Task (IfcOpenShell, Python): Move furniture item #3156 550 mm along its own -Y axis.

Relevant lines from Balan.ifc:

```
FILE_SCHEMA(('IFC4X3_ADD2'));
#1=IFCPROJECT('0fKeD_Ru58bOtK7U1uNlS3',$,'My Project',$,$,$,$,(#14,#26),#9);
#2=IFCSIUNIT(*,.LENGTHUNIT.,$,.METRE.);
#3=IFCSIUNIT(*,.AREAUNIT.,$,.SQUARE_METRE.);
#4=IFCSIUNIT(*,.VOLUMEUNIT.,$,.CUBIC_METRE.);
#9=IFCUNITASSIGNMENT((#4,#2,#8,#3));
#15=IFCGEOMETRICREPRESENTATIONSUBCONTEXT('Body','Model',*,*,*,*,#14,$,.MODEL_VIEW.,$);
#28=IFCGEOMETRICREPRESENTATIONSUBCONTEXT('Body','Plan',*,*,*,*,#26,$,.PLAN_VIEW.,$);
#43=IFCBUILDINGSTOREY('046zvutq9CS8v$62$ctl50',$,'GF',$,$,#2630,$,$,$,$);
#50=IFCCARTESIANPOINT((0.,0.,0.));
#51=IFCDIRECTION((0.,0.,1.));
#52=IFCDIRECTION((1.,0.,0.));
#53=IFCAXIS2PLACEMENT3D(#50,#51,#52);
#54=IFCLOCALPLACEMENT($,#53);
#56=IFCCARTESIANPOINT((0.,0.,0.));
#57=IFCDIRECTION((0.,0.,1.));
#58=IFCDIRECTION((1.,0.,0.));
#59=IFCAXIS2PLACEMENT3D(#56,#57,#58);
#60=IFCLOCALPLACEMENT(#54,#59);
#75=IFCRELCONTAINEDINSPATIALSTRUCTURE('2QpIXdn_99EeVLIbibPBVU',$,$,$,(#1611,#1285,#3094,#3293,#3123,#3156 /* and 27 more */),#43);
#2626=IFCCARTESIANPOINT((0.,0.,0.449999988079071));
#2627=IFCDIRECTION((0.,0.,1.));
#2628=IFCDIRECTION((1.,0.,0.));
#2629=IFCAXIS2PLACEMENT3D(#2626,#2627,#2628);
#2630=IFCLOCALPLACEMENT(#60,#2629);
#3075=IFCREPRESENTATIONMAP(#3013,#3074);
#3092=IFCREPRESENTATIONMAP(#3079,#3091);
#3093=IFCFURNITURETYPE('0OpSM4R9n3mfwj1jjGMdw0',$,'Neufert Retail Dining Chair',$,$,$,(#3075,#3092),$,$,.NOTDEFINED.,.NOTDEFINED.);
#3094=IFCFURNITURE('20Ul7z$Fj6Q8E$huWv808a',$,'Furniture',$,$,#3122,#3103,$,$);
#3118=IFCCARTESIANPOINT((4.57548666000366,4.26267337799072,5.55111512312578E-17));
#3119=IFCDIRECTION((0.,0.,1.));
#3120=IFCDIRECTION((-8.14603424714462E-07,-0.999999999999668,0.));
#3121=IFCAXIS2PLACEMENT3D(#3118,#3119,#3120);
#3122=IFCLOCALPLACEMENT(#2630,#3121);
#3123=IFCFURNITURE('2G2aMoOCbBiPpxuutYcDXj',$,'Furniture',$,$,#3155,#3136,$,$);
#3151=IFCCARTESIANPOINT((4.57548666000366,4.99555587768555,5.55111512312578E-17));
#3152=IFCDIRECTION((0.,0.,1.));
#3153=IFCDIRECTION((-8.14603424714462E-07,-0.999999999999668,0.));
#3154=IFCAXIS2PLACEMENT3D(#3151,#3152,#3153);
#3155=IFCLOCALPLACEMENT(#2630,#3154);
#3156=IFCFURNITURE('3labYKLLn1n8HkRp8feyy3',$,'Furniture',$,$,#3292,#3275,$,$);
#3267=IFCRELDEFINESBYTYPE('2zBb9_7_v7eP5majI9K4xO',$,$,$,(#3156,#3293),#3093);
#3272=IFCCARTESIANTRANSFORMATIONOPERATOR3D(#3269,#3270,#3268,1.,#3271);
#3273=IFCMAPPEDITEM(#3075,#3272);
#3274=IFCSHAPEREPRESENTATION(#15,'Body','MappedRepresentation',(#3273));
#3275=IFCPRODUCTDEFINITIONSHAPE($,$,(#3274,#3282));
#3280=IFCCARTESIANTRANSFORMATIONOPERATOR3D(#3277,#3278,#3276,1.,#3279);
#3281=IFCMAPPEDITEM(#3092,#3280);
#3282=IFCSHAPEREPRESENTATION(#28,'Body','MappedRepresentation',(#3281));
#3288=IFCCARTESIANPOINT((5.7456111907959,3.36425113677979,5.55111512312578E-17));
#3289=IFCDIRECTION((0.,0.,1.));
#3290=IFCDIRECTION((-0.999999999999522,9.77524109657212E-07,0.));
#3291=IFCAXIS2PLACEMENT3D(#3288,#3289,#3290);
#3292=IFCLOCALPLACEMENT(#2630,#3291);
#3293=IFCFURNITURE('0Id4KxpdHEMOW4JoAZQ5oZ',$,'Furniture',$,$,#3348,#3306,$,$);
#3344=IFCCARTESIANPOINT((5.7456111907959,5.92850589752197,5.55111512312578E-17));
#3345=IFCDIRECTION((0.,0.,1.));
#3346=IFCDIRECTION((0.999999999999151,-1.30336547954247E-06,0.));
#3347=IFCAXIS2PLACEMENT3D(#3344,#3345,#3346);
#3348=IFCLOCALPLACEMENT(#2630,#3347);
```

```python
import ifcopenshell
import ifcopenshell.api.geometry
import ifcopenshell.util.placement
import ifcopenshell.util.unit

model = ifcopenshell.open("Balan.ifc")
unit_scale = ifcopenshell.util.unit.calculate_unit_scale(model)

item = model.by_id(3156)
matrix = ifcopenshell.util.placement.get_local_placement(item.ObjectPlacement)
matrix[:3, 3] -= matrix[:3, 1] * 0.55 / unit_scale
ifcopenshell.api.geometry.edit_object_placement(model, product=item, matrix=matrix, is_si=False)

print(ifcopenshell.util.placement.get_local_placement(item.ObjectPlacement).round(3) + 0.0)

model.write("Balan_v2.ifc")
```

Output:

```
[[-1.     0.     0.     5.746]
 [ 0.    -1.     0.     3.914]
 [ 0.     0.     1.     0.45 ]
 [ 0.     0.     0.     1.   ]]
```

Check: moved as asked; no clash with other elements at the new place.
